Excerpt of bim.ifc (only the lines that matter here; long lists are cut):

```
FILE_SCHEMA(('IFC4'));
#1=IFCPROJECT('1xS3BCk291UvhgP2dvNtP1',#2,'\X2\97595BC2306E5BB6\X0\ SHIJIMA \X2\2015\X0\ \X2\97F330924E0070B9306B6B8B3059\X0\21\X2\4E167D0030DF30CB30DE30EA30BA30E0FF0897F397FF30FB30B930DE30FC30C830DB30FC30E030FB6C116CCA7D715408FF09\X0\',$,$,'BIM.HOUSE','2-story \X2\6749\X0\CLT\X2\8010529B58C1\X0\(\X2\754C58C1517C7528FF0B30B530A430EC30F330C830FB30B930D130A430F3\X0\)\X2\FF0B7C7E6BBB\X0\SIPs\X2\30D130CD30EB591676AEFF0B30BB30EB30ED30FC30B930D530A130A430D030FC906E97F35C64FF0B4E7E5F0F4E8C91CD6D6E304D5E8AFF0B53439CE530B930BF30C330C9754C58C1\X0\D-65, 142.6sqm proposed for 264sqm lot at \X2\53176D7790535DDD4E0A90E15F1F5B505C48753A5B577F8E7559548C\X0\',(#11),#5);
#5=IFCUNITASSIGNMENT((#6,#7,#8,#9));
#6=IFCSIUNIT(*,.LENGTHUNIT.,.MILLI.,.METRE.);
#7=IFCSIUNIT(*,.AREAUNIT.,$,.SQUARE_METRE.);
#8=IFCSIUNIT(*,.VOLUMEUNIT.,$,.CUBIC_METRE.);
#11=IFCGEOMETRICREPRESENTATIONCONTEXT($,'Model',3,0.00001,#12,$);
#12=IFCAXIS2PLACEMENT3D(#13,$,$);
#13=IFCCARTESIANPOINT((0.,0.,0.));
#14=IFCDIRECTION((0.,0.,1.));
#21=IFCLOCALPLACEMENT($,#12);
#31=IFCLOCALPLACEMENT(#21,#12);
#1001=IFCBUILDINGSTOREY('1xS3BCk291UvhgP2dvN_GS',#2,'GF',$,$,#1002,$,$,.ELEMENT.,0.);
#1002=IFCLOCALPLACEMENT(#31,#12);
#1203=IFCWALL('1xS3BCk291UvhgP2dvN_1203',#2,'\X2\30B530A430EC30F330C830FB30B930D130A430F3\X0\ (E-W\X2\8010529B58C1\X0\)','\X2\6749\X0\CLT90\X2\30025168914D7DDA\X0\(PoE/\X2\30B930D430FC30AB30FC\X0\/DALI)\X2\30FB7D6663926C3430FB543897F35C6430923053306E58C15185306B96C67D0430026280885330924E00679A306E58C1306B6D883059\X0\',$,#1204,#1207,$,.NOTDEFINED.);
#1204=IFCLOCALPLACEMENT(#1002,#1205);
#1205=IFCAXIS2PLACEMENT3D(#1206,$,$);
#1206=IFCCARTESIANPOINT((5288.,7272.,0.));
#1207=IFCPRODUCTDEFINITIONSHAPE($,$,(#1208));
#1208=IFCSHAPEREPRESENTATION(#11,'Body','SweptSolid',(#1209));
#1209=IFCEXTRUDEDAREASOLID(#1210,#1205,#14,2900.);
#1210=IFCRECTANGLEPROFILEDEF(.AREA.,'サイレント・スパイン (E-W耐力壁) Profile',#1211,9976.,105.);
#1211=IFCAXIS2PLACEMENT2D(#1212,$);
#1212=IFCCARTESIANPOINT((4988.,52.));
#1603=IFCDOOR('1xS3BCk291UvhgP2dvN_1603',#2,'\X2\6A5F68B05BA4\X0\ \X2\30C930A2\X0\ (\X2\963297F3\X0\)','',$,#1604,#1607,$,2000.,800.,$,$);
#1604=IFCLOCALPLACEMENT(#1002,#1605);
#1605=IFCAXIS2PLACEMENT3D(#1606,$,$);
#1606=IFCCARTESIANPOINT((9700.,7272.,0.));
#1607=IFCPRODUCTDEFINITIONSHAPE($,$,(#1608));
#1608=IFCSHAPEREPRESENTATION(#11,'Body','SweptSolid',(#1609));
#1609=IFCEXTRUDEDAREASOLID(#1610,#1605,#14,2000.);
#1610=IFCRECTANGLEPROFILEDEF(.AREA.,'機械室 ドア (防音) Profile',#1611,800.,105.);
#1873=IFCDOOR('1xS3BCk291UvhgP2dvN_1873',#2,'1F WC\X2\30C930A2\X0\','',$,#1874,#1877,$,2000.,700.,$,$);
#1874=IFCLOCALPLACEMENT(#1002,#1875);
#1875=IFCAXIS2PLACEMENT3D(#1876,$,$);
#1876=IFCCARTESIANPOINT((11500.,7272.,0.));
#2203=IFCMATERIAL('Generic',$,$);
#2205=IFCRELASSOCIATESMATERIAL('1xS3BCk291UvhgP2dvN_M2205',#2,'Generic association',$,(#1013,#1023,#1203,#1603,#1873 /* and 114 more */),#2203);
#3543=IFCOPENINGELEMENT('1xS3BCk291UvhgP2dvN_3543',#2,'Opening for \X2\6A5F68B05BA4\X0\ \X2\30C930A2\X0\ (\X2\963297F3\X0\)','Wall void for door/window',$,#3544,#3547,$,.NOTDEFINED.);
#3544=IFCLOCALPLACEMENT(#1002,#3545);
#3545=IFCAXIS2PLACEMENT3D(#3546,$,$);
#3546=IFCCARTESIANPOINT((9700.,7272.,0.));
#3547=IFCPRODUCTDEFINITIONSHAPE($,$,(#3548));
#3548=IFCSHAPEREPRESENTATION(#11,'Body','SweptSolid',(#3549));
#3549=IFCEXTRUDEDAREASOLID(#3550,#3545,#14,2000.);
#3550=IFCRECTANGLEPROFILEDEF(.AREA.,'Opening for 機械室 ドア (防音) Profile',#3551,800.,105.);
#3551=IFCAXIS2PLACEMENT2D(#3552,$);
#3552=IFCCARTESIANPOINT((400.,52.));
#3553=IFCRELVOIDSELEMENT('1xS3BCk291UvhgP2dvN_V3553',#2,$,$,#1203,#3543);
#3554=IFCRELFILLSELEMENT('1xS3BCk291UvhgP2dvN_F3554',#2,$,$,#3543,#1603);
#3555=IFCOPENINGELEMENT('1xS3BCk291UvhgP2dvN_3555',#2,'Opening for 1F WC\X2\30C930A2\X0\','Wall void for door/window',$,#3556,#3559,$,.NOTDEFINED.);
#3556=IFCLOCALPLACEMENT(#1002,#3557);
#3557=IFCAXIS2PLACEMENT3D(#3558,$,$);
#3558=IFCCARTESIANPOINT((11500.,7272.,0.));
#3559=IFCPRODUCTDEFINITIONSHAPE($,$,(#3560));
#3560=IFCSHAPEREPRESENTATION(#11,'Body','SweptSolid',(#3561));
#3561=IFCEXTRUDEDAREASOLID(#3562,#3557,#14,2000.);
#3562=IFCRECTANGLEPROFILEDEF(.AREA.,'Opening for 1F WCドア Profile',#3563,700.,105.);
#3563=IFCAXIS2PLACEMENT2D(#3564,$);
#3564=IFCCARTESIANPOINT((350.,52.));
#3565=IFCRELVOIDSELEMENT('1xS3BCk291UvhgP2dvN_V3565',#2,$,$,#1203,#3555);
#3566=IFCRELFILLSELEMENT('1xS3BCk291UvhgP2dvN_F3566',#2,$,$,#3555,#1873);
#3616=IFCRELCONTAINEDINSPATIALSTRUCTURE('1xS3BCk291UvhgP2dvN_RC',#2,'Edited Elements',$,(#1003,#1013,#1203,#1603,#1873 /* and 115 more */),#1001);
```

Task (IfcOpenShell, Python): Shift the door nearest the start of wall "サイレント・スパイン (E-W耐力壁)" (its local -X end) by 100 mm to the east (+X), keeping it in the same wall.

```python
import ifcopenshell
import ifcopenshell.api.geometry
import ifcopenshell.util.placement
import ifcopenshell.util.unit

model = ifcopenshell.open("bim.ifc")
unit_scale = ifcopenshell.util.unit.calculate_unit_scale(model)

door = model.by_guid("1xS3BCk291UvhgP2dvN_1603")
opening = door.FillsVoids[0].RelatingOpeningElement
wall = opening.VoidsElements[0].RelatingBuildingElement

wall_matrix = ifcopenshell.util.placement.get_local_placement(wall.ObjectPlacement)
shift = wall_matrix[:3, 0] * 0.1 / unit_scale
before = ifcopenshell.util.placement.get_local_placement(door.ObjectPlacement)[:3, 3].copy()

# The door is not placed relative to its opening, so move both.
for product in (opening, door):
    matrix = ifcopenshell.util.placement.get_local_placement(product.ObjectPlacement)
    matrix[:3, 3] += shift
    ifcopenshell.api.geometry.edit_object_placement(model, product=product, matrix=matrix, is_si=False)

after = ifcopenshell.util.placement.get_local_placement(door.ObjectPlacement)[:3, 3]
print("door moved by", (after - before).round(3) + 0.0)

model.write("bim_rev.ifc")
```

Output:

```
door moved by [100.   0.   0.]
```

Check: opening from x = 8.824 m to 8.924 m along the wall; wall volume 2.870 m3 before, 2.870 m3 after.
